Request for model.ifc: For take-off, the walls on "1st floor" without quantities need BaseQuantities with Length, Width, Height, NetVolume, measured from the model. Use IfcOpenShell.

First a look at what the model holds.

```python
import ifcopenshell
import ifcopenshell.util.element
import ifcopenshell.util.unit

model = ifcopenshell.open("model.ifc")
print(model.schema)
for unit_type in ("LENGTHUNIT", "AREAUNIT", "VOLUMEUNIT"):
    print(unit_type, ifcopenshell.util.unit.calculate_unit_scale(model, unit_type))
storey = next(s for s in model.by_type("IfcBuildingStorey") if s.Name == "1st floor")
walls = [e for e in ifcopenshell.util.element.get_decomposition(storey) if e.is_a("IfcWall")]
for e in sorted(walls, key=lambda e: e.id()):
    print(e.id(), e.is_a(), e.Name, list(ifcopenshell.util.element.get_psets(e, qtos_only=True)), sep=" | ")
```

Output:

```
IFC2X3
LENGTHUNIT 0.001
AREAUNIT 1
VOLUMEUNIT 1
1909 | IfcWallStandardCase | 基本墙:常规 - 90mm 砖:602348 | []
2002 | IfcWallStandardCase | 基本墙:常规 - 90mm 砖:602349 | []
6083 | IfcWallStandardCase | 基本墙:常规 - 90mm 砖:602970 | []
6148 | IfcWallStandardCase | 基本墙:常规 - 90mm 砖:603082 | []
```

```python
import ifcopenshell
import ifcopenshell.api.pset
import ifcopenshell.geom
import ifcopenshell.util.element
import ifcopenshell.util.shape
import ifcopenshell.util.unit

model = ifcopenshell.open("model.ifc")
unit_scale = ifcopenshell.util.unit.calculate_unit_scale(model)
volume_scale = ifcopenshell.util.unit.calculate_unit_scale(model, "VOLUMEUNIT")
settings = ifcopenshell.geom.settings()

storey = next(s for s in model.by_type("IfcBuildingStorey") if s.Name == "1st floor")
walls = [e for e in ifcopenshell.util.element.get_decomposition(storey) if e.is_a("IfcWall")]

for e in sorted(walls, key=lambda e: e.id()):
    if ifcopenshell.util.element.get_psets(e, qtos_only=True, should_inherit=False):
        continue
    # Geometry comes back in metres, in the element's own axes.
    shape = ifcopenshell.geom.create_shape(settings, e)
    values = {
        "Length": ifcopenshell.util.shape.get_x(shape.geometry) / unit_scale,
        "Width": ifcopenshell.util.shape.get_y(shape.geometry) / unit_scale,
        "Height": ifcopenshell.util.shape.get_z(shape.geometry) / unit_scale,
        "NetVolume": ifcopenshell.util.shape.get_volume(shape.geometry) / volume_scale,
    }
    qto = ifcopenshell.api.pset.add_qto(model, product=e, name="BaseQuantities")
    ifcopenshell.api.pset.edit_qto(model, qto=qto, properties=values)
    print(e.id(), {k: round(v, 3) for k, v in values.items()})

model.write("model_updated.ifc")
```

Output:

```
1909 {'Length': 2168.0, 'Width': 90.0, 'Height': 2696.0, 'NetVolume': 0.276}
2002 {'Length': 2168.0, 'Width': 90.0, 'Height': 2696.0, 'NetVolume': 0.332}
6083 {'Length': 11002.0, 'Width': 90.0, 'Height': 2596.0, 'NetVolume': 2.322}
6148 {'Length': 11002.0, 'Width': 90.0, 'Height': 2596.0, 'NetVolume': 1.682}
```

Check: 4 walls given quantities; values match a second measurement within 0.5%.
